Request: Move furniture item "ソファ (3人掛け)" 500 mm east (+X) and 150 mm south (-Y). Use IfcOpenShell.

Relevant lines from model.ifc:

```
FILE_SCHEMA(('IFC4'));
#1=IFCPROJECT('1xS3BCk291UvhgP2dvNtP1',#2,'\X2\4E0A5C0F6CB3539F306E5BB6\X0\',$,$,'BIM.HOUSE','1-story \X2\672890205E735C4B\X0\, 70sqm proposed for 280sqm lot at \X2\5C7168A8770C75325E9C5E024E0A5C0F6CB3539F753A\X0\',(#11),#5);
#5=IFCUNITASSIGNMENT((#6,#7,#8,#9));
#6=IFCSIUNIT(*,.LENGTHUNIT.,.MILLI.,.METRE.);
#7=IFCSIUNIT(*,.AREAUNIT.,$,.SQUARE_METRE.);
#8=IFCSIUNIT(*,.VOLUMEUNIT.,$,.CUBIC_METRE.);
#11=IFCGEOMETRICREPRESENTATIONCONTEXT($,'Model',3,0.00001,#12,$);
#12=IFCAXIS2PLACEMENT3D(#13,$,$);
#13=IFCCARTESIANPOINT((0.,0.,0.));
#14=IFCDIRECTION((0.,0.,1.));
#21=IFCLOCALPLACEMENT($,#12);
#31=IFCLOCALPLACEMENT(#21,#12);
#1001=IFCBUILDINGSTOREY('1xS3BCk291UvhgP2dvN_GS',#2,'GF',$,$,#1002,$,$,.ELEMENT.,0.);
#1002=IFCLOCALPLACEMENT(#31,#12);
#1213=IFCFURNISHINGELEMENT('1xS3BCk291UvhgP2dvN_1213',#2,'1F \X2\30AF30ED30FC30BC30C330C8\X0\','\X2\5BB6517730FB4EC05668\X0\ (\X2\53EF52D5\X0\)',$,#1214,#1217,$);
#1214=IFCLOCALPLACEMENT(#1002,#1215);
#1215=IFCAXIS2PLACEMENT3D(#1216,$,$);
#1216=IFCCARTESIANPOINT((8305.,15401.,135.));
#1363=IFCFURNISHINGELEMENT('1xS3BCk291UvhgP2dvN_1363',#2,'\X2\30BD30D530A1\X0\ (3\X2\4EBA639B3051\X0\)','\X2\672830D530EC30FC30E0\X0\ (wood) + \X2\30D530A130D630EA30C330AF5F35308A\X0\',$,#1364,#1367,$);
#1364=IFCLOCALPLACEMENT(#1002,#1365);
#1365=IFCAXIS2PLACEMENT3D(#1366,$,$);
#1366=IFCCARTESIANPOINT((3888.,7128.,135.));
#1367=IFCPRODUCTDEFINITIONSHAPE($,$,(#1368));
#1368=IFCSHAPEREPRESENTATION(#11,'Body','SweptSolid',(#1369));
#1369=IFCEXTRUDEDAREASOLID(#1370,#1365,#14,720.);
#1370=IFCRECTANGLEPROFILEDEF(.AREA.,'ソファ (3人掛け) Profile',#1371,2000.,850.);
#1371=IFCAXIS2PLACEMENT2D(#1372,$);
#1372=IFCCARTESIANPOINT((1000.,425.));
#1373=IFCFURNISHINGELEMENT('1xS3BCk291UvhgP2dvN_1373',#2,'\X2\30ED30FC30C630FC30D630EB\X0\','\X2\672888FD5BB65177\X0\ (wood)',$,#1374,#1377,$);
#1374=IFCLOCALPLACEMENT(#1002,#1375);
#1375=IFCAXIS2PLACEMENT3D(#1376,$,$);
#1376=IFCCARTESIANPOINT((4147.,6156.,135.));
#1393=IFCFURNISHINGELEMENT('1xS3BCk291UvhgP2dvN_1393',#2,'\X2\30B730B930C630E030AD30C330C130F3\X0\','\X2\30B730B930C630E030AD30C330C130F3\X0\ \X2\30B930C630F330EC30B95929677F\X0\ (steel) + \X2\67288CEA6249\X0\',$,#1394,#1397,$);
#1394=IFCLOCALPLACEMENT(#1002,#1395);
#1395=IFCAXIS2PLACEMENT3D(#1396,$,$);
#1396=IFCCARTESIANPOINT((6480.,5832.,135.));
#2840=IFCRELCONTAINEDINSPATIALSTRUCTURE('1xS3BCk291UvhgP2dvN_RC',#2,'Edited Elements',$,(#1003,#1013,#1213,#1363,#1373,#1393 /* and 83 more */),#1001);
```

```python
import ifcopenshell
import ifcopenshell.api.geometry
import ifcopenshell.util.placement
import ifcopenshell.util.unit

model = ifcopenshell.open("model.ifc")
unit_scale = ifcopenshell.util.unit.calculate_unit_scale(model)

item = model.by_id(1363)
matrix = ifcopenshell.util.placement.get_local_placement(item.ObjectPlacement)
matrix[0, 3] += 0.5 / unit_scale
matrix[1, 3] -= 0.15 / unit_scale
ifcopenshell.api.geometry.edit_object_placement(model, product=item, matrix=matrix, is_si=False)

print(ifcopenshell.util.placement.get_local_placement(item.ObjectPlacement).round(3) + 0.0)

model.write("model_rev.ifc")
```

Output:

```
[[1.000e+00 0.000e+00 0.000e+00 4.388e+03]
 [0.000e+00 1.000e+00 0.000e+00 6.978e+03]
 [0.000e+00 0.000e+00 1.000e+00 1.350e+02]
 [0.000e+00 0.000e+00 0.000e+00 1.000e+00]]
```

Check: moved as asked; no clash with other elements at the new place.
